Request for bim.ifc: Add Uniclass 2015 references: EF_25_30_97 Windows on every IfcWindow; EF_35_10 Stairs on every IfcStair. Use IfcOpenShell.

First a look at what the model holds.

```python
import ifcopenshell

model = ifcopenshell.open("bim.ifc")
print(model.schema)
print("classifications:", [c.Name for c in model.by_type("IfcClassification")])
for ifc_class in ("IfcDoor", "IfcRoof", "IfcStair", "IfcWall", "IfcWindow"):
    print(ifc_class, len(model.by_type(ifc_class)))
```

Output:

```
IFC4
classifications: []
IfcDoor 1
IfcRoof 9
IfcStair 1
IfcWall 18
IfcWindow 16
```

```python
import ifcopenshell
import ifcopenshell.api.classification

model = ifcopenshell.open("bim.ifc")

system = ifcopenshell.api.classification.add_classification(model, classification="Uniclass 2015")

codes = {
    "IfcWindow": ("EF_25_30_97", "Windows"),
    "IfcStair": ("EF_35_10", "Stairs"),
}
for ifc_class, (code, name) in codes.items():
    products = model.by_type(ifc_class)
    ifcopenshell.api.classification.add_reference(
        model, products=products, classification=system, identification=code, name=name
    )
    print(code, len(products))

model.write("bim_updated.ifc")
```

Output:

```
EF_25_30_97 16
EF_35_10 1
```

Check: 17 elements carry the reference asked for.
